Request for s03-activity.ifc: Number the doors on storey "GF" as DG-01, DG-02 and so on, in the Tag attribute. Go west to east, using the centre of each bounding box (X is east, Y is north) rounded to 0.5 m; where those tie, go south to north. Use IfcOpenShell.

First a look at what the model holds.

```python
import ifcopenshell
import ifcopenshell.util.element
import ifcopenshell.util.placement

model = ifcopenshell.open("s03-activity.ifc")
print(model.schema)
storey = next(s for s in model.by_type("IfcBuildingStorey") if s.Name == "GF")
doors = [e for e in ifcopenshell.util.element.get_decomposition(storey) if e.is_a("IfcDoor")]
for e in sorted(doors, key=lambda e: e.id()):
    origin = ifcopenshell.util.placement.get_local_placement(e.ObjectPlacement)[:3, 3]
    print(e.id(), e.Tag, e.Name, origin.round(2) + 0.0, sep=" | ")
```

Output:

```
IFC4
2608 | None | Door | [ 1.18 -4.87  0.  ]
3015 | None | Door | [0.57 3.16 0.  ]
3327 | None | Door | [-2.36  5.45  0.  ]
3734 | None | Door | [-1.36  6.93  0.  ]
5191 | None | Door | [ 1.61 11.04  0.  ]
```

```python
import ifcopenshell
import ifcopenshell.geom
import ifcopenshell.util.element
import ifcopenshell.util.shape

model = ifcopenshell.open("s03-activity.ifc")
settings = ifcopenshell.geom.settings()
settings.set("use-world-coords", True)


def centre(element):
    shape = ifcopenshell.geom.create_shape(settings, element)
    return ifcopenshell.util.shape.get_bbox_centroid(shape.geometry)


storey = next(s for s in model.by_type("IfcBuildingStorey") if s.Name == "GF")
doors = [e for e in ifcopenshell.util.element.get_decomposition(storey) if e.is_a("IfcDoor")]

# Insertion points can sit at a corner or the storey origin, so sort by the geometry (in metres).
centres = {e: centre(e) for e in doors}
doors.sort(key=lambda e: (round(centres[e][0] / 0.5), centres[e][1]))

for i, e in enumerate(doors, start=1):
    number = f"DG-{i:02d}"
    e.Tag = number
    print(e.id(), number)

model.write("s03-activity-out.ifc")
```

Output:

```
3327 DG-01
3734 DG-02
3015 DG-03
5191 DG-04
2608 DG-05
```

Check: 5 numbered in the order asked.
